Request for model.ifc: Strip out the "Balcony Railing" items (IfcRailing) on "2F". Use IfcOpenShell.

First a look at what the model holds.

```python
import ifcopenshell
import ifcopenshell.util.element

model = ifcopenshell.open("model.ifc")
print(model.schema)
storey = next(s for s in model.by_type("IfcBuildingStorey") if s.Name == "2F")
railings = [e for e in ifcopenshell.util.element.get_decomposition(storey) if e.is_a("IfcRailing")]
seen = {}
for e in railings:
    element_type = ifcopenshell.util.element.get_type(e)
    name = element_type.Name if element_type not in (None, e) else None
    seen[name] = seen.get(name, 0) + 1
for name, count in sorted(seen.items(), key=str):
    print(count, "x", name)
```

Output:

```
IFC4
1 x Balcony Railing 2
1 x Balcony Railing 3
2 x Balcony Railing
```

```python
import ifcopenshell
import ifcopenshell.api.root
import ifcopenshell.util.element

model = ifcopenshell.open("model.ifc")

storey = next(s for s in model.by_type("IfcBuildingStorey") if s.Name == "2F")
railings = [e for e in ifcopenshell.util.element.get_decomposition(storey) if e.is_a("IfcRailing")]
targets = [e for e in railings if (t := ifcopenshell.util.element.get_type(e)) not in (None, e) and t.Name == "Balcony Railing"]

for e in targets:
    ifcopenshell.api.root.remove_product(model, product=e)
print(len(targets), "removed")

model.write("model_edited.ifc")
```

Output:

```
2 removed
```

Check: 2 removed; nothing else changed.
